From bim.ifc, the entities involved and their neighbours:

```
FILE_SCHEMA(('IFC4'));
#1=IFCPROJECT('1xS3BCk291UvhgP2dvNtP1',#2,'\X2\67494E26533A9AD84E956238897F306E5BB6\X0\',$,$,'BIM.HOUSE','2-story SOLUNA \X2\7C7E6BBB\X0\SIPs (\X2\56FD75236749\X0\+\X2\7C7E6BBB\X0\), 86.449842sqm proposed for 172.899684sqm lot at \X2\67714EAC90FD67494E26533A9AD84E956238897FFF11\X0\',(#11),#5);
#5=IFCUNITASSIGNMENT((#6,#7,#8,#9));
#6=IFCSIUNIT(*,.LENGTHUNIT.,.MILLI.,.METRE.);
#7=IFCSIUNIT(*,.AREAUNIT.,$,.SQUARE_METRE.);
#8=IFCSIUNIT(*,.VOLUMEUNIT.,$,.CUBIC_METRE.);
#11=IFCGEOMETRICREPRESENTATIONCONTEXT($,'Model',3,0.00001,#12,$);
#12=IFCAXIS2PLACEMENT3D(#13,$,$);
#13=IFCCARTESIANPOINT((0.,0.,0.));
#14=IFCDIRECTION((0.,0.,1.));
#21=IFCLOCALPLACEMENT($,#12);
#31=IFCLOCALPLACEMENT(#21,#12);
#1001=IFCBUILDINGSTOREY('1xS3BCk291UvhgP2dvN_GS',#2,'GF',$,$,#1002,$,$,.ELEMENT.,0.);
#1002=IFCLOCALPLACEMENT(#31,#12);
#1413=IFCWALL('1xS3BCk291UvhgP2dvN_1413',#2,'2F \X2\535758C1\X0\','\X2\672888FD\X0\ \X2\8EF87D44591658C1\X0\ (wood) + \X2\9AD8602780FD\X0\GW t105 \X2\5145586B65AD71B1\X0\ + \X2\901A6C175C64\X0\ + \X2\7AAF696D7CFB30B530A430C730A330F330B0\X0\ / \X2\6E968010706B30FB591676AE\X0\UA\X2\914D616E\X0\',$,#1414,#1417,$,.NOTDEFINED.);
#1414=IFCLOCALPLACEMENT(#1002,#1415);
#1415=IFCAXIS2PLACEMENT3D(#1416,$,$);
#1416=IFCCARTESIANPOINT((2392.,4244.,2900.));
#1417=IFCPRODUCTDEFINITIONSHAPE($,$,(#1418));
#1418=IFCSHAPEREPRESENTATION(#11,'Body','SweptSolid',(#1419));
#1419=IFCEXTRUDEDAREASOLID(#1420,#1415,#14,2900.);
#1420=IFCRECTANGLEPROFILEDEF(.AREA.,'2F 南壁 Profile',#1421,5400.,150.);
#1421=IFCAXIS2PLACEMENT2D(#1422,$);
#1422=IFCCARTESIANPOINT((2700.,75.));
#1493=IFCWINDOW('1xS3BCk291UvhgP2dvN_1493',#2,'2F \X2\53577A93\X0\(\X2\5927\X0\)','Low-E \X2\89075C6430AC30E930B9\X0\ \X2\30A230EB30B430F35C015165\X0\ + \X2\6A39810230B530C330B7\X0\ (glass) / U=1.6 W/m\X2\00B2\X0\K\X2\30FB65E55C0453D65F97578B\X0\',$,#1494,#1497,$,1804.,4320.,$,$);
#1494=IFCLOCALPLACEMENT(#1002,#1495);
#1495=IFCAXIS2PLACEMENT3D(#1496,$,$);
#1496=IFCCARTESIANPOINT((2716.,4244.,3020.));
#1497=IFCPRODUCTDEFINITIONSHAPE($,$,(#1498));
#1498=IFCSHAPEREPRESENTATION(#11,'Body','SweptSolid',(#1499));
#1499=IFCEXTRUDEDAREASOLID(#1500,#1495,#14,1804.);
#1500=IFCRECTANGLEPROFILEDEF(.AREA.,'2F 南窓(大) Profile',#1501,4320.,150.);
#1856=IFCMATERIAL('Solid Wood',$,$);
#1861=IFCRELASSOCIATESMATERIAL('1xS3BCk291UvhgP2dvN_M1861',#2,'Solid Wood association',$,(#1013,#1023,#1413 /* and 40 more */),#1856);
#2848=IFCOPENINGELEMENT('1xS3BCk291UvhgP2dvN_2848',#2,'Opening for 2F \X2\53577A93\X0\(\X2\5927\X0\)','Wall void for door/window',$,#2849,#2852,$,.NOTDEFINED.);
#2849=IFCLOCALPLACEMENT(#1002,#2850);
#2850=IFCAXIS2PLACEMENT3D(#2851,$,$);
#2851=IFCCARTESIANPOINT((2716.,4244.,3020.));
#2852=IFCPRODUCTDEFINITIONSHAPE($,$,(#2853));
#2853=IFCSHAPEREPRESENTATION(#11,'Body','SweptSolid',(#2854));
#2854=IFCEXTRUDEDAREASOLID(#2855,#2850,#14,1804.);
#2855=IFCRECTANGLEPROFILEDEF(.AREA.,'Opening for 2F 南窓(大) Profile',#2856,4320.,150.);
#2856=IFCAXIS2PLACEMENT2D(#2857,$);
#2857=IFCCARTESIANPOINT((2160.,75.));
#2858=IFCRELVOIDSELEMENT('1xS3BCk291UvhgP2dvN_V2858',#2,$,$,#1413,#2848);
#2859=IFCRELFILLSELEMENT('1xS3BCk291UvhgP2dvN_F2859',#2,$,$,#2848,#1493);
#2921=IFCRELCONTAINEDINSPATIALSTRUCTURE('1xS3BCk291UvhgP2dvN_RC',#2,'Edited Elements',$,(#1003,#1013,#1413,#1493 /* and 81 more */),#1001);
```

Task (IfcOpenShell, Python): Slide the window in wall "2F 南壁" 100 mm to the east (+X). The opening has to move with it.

```python
import ifcopenshell
import ifcopenshell.api.geometry
import ifcopenshell.util.placement

model = ifcopenshell.open("bim.ifc")

window = model.by_guid("1xS3BCk291UvhgP2dvN_1493")
opening = window.FillsVoids[0].RelatingOpeningElement
wall = opening.VoidsElements[0].RelatingBuildingElement

wall_matrix = ifcopenshell.util.placement.get_local_placement(wall.ObjectPlacement)
shift = wall_matrix[:3, 0] * 100.0
before = ifcopenshell.util.placement.get_local_placement(window.ObjectPlacement)[:3, 3].copy()

# The window is not placed relative to its opening, so move both.
for product in (opening, window):
    matrix = ifcopenshell.util.placement.get_local_placement(product.ObjectPlacement)
    matrix[:3, 3] += shift
    ifcopenshell.api.geometry.edit_object_placement(model, product=product, matrix=matrix, is_si=False)

after = ifcopenshell.util.placement.get_local_placement(window.ObjectPlacement)[:3, 3]
print("window moved by", (after - before).round(3) + 0.0)

model.write("bim_updated.ifc")
```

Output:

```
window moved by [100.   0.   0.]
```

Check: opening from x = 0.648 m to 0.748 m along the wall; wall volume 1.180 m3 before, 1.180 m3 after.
